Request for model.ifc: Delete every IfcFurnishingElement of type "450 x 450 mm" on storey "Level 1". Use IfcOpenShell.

First a look at what the model holds.

```python
import ifcopenshell
import ifcopenshell.util.element

model = ifcopenshell.open("model.ifc")
print(model.schema)
storey = next(s for s in model.by_type("IfcBuildingStorey") if s.Name == "Level 1")
furniture = [e for e in ifcopenshell.util.element.get_decomposition(storey) if e.is_a("IfcFurnishingElement")]
seen = {}
for e in furniture:
    element_type = ifcopenshell.util.element.get_type(e)
    name = element_type.Name if element_type not in (None, e) else None
    seen[name] = seen.get(name, 0) + 1
for name, count in sorted(seen.items(), key=str):
    print(count, "x", name)
```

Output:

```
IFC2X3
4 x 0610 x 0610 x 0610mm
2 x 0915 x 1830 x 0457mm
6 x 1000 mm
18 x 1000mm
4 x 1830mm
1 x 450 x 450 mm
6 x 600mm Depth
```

```python
import ifcopenshell
import ifcopenshell.api.root
import ifcopenshell.util.element

model = ifcopenshell.open("model.ifc")

storey = next(s for s in model.by_type("IfcBuildingStorey") if s.Name == "Level 1")
furniture = [e for e in ifcopenshell.util.element.get_decomposition(storey) if e.is_a("IfcFurnishingElement")]
targets = [e for e in furniture if (t := ifcopenshell.util.element.get_type(e)) not in (None, e) and t.Name == "450 x 450 mm"]

for e in targets:
    ifcopenshell.api.root.remove_product(model, product=e)
print(len(targets), "removed")

model.write("model-out.ifc")
```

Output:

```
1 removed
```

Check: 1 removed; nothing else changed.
